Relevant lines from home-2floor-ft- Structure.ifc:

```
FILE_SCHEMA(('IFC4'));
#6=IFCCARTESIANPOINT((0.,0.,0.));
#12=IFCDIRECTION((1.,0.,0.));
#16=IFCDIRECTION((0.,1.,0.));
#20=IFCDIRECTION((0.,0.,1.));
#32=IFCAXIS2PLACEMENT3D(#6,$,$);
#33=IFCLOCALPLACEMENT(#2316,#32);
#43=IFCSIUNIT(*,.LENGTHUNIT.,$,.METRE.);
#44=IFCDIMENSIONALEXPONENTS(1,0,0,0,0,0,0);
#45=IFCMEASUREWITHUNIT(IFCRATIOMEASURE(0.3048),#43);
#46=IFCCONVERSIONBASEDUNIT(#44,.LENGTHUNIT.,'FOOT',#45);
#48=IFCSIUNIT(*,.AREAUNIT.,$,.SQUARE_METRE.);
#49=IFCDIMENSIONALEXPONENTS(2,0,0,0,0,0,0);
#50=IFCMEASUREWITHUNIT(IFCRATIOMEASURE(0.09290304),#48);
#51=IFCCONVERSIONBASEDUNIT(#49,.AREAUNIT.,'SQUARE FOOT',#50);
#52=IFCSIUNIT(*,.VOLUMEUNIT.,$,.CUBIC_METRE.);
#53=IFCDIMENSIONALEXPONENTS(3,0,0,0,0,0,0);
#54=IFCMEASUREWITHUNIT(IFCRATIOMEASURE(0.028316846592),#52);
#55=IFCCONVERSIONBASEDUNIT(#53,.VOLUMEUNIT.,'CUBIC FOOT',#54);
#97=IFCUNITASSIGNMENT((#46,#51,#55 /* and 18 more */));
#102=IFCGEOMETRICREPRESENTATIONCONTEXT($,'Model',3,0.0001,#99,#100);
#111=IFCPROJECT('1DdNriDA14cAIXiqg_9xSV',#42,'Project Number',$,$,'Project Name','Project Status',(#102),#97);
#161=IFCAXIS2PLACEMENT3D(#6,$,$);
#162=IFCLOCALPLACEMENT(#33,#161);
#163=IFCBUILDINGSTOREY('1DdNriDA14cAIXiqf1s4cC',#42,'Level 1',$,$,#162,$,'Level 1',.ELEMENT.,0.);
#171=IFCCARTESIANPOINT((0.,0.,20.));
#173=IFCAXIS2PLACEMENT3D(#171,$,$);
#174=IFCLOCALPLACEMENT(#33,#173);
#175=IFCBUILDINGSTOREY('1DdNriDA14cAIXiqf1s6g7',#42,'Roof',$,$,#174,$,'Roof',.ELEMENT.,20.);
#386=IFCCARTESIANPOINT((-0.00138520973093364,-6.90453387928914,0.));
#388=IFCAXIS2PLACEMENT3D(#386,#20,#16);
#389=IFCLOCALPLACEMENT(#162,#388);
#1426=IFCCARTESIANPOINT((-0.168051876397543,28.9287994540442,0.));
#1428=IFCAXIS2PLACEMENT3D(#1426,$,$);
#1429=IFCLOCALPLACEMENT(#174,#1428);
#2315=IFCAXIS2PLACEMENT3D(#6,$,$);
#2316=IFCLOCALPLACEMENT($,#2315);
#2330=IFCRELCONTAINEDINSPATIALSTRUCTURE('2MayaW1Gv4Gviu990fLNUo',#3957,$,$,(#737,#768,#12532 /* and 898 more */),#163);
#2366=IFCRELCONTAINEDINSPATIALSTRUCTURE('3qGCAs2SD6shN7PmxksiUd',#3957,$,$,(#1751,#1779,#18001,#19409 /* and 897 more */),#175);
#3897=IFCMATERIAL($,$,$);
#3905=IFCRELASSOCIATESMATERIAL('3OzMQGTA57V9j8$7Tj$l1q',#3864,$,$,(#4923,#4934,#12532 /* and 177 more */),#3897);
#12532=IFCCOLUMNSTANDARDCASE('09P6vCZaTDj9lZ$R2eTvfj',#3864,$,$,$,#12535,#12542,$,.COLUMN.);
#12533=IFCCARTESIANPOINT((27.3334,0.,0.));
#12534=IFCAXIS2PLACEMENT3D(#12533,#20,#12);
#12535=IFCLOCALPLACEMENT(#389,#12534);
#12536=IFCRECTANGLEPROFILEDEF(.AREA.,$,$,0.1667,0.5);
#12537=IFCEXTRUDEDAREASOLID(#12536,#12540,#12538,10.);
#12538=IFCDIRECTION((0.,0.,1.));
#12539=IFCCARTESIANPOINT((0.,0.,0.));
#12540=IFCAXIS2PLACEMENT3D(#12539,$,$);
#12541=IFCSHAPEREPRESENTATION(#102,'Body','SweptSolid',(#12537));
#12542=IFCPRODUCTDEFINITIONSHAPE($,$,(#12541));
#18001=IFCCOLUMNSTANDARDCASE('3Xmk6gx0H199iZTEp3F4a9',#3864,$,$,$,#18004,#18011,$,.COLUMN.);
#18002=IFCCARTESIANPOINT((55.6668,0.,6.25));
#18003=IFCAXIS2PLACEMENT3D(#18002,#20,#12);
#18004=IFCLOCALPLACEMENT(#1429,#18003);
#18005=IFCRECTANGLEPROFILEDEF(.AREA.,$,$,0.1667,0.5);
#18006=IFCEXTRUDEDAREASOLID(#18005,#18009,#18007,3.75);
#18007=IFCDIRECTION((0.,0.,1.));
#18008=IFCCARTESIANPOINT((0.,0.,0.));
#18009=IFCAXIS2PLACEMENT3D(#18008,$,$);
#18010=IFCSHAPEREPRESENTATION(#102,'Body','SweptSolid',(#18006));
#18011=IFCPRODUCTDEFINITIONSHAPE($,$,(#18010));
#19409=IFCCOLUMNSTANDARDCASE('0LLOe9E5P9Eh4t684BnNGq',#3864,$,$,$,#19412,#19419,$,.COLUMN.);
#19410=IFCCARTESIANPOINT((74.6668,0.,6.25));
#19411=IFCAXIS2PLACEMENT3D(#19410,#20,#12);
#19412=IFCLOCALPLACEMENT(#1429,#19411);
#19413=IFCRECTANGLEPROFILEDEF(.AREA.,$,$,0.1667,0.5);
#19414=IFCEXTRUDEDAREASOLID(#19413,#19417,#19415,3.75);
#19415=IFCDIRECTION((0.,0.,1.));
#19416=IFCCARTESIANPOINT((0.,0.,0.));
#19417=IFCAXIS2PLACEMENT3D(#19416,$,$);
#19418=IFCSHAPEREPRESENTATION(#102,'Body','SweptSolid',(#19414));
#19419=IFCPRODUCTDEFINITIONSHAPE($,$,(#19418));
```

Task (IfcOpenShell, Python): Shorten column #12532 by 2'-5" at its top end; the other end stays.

```python
import ifcopenshell
import ifcopenshell.util.unit

model = ifcopenshell.open("home-2floor-ft- Structure.ifc")
unit_scale = ifcopenshell.util.unit.calculate_unit_scale(model)

member = model.by_guid("09P6vCZaTDj9lZ$R2eTvfj")
change = -29 * 0.0254 / unit_scale

# The extrusion runs towards the end named, so only its depth changes.
body = next(r for r in member.Representation.Representations if r.RepresentationIdentifier == "Body")
solid = body.Items[0]
old_length = solid.Depth
solid.Depth += change

print(f"length {old_length:g} -> {solid.Depth:g}")

model.write("home-2floor-ft- Structure_edited.ifc")
```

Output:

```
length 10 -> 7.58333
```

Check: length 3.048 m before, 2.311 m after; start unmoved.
